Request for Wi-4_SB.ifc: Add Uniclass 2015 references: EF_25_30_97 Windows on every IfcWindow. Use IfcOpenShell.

First a look at what the model holds.

```python
import ifcopenshell

model = ifcopenshell.open("Wi-4_SB.ifc")
print(model.schema)
print("classifications:", [c.Name for c in model.by_type("IfcClassification")])
for ifc_class in ("IfcDoor", "IfcRoof", "IfcStair", "IfcWall", "IfcWindow"):
    print(ifc_class, len(model.by_type(ifc_class)))
```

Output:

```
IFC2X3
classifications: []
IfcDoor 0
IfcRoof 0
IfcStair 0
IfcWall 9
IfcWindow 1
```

```python
import ifcopenshell
import ifcopenshell.api.classification

model = ifcopenshell.open("Wi-4_SB.ifc")

# IFC2X3 requires Source and Edition and has no link from the project to the system.
system = model.create_entity("IfcClassification", Source="NBS", Edition="2015", Name="Uniclass 2015")

codes = {
    "IfcWindow": ("EF_25_30_97", "Windows"),
}
for ifc_class, (code, name) in codes.items():
    products = model.by_type(ifc_class)
    ifcopenshell.api.classification.add_reference(
        model, products=products, classification=system, identification=code, name=name
    )
    print(code, len(products))

model.write("Wi-4_SB-out.ifc")
```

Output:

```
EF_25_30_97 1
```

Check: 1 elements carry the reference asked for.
